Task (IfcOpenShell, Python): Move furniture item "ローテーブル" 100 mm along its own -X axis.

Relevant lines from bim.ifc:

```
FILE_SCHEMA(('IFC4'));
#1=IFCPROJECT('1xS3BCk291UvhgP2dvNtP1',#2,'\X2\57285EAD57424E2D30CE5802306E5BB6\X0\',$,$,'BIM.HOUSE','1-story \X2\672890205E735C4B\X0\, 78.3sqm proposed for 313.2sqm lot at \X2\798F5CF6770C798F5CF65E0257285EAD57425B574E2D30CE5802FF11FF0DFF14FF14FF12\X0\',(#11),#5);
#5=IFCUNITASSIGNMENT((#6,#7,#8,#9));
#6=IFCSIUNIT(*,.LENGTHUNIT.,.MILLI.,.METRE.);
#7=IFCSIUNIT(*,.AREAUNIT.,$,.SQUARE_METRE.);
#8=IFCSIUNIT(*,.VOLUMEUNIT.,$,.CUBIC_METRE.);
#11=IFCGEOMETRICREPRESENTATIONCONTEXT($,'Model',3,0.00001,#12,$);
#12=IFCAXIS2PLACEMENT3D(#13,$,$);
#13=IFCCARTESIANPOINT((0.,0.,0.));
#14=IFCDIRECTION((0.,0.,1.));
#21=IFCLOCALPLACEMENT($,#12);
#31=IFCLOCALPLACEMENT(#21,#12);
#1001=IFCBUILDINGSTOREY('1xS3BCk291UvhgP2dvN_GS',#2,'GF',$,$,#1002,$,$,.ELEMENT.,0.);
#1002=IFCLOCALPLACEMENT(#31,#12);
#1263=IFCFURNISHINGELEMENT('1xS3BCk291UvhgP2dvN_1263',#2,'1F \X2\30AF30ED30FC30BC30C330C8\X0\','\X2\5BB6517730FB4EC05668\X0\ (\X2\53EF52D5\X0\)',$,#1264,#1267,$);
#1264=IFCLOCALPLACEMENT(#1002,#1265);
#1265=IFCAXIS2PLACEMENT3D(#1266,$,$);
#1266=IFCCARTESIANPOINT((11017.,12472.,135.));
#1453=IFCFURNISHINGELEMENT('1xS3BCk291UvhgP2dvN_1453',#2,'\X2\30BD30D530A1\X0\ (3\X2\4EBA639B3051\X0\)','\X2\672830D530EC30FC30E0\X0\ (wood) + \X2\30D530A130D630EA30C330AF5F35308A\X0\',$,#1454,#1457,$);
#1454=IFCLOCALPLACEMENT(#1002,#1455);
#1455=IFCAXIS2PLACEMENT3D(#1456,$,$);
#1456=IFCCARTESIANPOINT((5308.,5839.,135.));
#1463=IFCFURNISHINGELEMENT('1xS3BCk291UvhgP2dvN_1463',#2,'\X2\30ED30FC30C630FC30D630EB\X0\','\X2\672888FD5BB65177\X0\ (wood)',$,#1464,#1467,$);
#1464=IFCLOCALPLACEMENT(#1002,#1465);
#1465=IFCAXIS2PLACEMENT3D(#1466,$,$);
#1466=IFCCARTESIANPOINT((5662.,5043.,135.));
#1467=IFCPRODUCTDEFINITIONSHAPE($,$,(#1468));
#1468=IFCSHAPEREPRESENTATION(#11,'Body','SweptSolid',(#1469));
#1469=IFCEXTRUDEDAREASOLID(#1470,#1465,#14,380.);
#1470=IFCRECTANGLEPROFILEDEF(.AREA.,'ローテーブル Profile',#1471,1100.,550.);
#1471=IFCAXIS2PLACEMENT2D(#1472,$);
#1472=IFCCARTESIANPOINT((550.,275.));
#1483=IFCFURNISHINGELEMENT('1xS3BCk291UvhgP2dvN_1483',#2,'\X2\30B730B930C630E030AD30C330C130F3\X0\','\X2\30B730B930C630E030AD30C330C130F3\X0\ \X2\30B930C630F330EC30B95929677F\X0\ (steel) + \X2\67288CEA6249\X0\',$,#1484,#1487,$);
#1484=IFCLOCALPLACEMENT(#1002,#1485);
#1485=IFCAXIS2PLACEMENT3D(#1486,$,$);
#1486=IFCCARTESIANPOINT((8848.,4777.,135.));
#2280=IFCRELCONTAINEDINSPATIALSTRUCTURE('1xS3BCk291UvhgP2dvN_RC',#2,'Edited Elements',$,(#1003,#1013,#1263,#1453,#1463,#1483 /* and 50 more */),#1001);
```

```python
import ifcopenshell
import ifcopenshell.api.geometry
import ifcopenshell.util.placement
import ifcopenshell.util.unit

model = ifcopenshell.open("bim.ifc")
unit_scale = ifcopenshell.util.unit.calculate_unit_scale(model)

item = model.by_id(1463)
matrix = ifcopenshell.util.placement.get_local_placement(item.ObjectPlacement)
matrix[:3, 3] -= matrix[:3, 0] * 0.1 / unit_scale
ifcopenshell.api.geometry.edit_object_placement(model, product=item, matrix=matrix, is_si=False)

print(ifcopenshell.util.placement.get_local_placement(item.ObjectPlacement).round(3) + 0.0)

model.write("bim_updated.ifc")
```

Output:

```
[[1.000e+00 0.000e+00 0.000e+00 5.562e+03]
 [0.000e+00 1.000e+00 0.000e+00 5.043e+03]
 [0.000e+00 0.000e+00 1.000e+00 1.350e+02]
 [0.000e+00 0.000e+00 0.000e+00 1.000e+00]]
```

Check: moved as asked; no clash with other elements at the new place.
